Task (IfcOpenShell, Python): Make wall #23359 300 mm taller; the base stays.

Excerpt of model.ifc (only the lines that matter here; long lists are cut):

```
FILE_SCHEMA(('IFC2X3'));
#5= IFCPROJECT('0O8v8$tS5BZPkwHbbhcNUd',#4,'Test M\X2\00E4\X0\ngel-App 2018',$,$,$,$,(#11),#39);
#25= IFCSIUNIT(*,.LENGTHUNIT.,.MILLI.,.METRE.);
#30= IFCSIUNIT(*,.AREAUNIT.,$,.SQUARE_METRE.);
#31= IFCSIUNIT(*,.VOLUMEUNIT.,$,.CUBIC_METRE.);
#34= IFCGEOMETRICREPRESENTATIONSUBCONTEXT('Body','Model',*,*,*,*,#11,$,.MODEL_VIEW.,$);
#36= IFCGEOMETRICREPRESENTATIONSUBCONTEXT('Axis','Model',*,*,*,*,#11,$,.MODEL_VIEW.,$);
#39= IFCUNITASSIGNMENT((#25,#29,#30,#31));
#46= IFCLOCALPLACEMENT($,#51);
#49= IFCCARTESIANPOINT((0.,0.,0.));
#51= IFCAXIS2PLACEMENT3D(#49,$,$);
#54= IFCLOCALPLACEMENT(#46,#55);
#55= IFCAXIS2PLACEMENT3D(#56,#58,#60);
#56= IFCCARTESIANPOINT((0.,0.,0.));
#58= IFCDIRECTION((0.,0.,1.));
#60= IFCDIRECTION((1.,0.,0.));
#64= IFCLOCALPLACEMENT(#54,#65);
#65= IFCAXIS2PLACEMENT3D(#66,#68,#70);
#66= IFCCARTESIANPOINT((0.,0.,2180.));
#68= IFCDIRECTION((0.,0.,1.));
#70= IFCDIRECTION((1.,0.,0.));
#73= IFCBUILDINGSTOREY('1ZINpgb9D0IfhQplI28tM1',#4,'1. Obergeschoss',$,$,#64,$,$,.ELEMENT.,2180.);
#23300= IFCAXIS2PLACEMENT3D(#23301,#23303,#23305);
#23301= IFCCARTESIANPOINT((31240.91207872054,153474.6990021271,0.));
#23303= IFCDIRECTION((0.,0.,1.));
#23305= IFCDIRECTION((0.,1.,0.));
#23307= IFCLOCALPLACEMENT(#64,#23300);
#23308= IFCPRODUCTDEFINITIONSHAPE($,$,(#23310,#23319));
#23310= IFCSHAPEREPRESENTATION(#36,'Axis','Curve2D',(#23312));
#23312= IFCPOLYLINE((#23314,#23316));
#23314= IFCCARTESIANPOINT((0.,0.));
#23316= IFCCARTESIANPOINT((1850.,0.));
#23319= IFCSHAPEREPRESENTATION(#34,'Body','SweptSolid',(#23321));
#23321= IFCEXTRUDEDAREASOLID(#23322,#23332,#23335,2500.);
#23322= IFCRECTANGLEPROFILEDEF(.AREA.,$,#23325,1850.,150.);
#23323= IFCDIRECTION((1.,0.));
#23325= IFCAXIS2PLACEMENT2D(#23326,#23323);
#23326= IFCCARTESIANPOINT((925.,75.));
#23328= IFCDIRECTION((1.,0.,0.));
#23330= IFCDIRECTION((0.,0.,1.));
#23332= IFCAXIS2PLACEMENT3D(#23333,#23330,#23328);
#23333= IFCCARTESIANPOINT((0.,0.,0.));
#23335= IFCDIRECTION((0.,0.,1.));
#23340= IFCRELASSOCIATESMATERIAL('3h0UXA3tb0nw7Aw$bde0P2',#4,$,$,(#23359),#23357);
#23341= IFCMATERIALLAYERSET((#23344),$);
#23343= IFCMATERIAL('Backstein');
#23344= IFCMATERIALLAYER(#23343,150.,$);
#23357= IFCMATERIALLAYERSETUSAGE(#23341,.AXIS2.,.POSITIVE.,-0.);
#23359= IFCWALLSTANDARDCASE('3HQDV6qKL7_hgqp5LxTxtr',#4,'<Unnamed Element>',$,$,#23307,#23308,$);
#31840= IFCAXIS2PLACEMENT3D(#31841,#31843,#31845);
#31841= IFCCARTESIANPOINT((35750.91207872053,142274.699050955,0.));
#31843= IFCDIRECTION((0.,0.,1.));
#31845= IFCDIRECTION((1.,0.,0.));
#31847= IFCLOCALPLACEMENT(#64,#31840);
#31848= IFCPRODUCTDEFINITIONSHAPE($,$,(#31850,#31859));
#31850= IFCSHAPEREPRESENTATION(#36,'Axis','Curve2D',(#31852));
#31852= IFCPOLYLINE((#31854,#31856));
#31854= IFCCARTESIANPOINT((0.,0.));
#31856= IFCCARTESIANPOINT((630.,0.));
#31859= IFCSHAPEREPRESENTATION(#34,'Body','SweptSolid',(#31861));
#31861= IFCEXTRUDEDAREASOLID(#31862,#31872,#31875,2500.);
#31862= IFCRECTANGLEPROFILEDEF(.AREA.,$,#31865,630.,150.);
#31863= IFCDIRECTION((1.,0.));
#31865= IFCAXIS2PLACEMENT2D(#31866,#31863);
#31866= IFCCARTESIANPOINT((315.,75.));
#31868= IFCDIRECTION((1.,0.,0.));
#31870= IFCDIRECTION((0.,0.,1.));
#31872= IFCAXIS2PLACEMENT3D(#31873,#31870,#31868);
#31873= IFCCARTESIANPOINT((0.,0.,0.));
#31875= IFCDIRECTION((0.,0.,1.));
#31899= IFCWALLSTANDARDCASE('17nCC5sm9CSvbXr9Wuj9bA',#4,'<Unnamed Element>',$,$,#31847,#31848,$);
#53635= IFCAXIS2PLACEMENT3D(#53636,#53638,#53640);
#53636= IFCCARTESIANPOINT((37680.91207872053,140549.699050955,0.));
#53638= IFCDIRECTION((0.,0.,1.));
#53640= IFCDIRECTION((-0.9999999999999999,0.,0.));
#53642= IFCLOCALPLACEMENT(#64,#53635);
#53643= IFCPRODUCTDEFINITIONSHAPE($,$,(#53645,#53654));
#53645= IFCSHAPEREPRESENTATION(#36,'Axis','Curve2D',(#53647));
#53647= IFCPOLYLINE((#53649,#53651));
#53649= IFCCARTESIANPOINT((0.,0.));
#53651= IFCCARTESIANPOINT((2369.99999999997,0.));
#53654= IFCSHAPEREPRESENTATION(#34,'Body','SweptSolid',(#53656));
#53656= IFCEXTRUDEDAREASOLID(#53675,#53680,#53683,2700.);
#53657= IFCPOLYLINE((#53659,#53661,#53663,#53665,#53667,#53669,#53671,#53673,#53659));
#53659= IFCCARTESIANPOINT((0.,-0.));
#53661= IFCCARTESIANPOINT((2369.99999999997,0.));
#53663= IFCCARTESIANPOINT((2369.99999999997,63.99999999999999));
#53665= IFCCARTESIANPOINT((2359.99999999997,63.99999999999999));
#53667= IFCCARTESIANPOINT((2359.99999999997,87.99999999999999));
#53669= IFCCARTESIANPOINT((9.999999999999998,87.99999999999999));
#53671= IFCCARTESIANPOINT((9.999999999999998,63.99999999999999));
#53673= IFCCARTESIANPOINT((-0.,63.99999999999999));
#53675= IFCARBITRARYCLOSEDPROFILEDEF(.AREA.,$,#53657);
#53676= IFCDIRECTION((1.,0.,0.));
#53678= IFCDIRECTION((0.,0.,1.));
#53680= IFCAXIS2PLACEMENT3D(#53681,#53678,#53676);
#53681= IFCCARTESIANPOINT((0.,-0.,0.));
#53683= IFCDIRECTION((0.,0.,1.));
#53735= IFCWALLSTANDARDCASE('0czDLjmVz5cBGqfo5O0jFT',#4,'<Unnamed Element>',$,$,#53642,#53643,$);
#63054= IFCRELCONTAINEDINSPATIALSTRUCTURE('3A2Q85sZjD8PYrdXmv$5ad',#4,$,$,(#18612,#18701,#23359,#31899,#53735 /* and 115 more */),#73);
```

```python
import ifcopenshell
import ifcopenshell.geom
import ifcopenshell.util.representation
import ifcopenshell.util.shape
import ifcopenshell.util.unit

model = ifcopenshell.open("model.ifc")
unit_scale = ifcopenshell.util.unit.calculate_unit_scale(model)
settings = ifcopenshell.geom.settings()


def volume(element):
    """Net volume in cubic metres, openings subtracted."""
    shape = ifcopenshell.geom.create_shape(settings, element)
    return ifcopenshell.util.shape.get_volume(shape.geometry)


wall = model.by_guid("3HQDV6qKL7_hgqp5LxTxtr")
before = volume(wall)

body = ifcopenshell.util.representation.get_representation(wall, "Model", "Body")
solid = body.Items[0]
old_height = solid.Depth
solid.Depth += 0.3 / unit_scale
after = volume(wall)

print(f"height {old_height:g} -> {solid.Depth:g}, volume {before:.3f} -> {after:.3f} m3")

model.write("model_edited.ifc")
```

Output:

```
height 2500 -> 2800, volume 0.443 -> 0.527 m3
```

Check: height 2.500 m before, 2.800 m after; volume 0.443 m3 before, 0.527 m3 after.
